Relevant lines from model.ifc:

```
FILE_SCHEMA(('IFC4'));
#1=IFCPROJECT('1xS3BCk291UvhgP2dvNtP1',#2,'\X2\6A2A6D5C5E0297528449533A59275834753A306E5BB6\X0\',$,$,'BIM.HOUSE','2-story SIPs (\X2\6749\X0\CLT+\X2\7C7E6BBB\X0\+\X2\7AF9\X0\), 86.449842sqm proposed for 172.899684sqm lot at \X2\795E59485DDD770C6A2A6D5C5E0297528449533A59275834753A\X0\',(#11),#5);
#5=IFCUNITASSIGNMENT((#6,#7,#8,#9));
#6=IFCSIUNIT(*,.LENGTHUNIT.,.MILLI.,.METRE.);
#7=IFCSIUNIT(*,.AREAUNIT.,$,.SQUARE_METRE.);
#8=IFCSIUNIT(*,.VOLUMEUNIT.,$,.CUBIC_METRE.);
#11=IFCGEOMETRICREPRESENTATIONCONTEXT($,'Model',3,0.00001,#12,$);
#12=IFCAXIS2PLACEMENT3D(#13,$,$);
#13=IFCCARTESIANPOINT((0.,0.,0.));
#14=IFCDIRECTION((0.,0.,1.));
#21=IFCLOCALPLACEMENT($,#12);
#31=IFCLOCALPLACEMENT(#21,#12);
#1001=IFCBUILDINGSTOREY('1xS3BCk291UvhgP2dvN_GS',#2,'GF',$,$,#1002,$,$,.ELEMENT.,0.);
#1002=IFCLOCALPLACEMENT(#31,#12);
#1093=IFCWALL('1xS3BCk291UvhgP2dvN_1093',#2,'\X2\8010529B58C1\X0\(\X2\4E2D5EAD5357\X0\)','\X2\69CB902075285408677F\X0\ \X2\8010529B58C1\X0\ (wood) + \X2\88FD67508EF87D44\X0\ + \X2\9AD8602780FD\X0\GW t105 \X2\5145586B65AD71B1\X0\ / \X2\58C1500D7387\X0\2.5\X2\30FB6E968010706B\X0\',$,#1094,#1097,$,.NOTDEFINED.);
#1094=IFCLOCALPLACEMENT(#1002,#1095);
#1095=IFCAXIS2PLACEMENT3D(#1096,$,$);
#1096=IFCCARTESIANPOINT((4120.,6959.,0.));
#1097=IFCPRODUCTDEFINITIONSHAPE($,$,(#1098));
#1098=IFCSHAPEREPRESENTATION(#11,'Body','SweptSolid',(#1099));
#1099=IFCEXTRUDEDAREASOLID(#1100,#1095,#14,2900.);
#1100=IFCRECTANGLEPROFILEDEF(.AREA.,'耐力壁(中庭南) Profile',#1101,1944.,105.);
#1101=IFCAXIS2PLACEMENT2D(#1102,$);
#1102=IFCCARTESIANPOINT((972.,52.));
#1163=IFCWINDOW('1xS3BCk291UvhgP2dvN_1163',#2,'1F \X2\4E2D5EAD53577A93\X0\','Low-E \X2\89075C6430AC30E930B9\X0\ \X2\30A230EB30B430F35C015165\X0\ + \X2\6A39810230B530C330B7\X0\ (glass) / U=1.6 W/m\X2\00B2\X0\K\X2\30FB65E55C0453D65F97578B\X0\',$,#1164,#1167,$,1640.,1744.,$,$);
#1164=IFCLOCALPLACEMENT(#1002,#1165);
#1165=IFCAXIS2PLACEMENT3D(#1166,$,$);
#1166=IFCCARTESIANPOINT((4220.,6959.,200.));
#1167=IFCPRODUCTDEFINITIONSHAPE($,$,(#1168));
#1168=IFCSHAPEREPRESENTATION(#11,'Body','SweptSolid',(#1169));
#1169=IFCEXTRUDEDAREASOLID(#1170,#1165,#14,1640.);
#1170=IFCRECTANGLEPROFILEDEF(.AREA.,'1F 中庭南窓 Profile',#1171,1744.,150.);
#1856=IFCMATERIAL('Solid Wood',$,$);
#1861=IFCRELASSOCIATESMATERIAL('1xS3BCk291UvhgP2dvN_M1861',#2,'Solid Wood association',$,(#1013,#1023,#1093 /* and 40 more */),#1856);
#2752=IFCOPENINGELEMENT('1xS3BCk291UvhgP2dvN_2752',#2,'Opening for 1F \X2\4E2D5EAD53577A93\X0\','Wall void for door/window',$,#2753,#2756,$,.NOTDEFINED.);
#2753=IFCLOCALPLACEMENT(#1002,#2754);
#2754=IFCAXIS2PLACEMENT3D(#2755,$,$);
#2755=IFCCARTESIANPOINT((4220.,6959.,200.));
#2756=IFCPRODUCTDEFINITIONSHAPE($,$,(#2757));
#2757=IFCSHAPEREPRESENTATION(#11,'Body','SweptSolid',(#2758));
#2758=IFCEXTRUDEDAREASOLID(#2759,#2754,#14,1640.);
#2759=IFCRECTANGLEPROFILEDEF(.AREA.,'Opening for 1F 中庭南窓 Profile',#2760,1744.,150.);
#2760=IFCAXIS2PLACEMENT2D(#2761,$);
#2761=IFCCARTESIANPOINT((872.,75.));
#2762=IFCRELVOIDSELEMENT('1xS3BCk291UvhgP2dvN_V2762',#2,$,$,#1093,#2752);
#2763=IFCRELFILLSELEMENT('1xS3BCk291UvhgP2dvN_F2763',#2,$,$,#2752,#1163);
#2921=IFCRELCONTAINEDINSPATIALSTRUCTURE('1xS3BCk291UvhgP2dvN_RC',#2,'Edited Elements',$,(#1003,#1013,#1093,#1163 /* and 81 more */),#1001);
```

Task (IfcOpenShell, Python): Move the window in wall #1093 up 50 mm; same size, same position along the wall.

```python
import numpy as np
import ifcopenshell
import ifcopenshell.api.geometry
import ifcopenshell.util.placement
import ifcopenshell.util.unit

model = ifcopenshell.open("model.ifc")
unit_scale = ifcopenshell.util.unit.calculate_unit_scale(model)

window = model.by_guid("1xS3BCk291UvhgP2dvN_1163")
opening = window.FillsVoids[0].RelatingOpeningElement
dz = 50.0

shift = np.array([0.0, 0.0, dz])
# The window is not placed relative to its opening, so move both.
for product in (opening, window):
    matrix = ifcopenshell.util.placement.get_local_placement(product.ObjectPlacement)
    matrix[:3, 3] += shift
    ifcopenshell.api.geometry.edit_object_placement(model, product=product, matrix=matrix, is_si=False)

print(f"moved by {dz * unit_scale:+.3f} m")

model.write("model_v2.ifc")
```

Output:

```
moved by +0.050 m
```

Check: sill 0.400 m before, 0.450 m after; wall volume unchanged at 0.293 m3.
